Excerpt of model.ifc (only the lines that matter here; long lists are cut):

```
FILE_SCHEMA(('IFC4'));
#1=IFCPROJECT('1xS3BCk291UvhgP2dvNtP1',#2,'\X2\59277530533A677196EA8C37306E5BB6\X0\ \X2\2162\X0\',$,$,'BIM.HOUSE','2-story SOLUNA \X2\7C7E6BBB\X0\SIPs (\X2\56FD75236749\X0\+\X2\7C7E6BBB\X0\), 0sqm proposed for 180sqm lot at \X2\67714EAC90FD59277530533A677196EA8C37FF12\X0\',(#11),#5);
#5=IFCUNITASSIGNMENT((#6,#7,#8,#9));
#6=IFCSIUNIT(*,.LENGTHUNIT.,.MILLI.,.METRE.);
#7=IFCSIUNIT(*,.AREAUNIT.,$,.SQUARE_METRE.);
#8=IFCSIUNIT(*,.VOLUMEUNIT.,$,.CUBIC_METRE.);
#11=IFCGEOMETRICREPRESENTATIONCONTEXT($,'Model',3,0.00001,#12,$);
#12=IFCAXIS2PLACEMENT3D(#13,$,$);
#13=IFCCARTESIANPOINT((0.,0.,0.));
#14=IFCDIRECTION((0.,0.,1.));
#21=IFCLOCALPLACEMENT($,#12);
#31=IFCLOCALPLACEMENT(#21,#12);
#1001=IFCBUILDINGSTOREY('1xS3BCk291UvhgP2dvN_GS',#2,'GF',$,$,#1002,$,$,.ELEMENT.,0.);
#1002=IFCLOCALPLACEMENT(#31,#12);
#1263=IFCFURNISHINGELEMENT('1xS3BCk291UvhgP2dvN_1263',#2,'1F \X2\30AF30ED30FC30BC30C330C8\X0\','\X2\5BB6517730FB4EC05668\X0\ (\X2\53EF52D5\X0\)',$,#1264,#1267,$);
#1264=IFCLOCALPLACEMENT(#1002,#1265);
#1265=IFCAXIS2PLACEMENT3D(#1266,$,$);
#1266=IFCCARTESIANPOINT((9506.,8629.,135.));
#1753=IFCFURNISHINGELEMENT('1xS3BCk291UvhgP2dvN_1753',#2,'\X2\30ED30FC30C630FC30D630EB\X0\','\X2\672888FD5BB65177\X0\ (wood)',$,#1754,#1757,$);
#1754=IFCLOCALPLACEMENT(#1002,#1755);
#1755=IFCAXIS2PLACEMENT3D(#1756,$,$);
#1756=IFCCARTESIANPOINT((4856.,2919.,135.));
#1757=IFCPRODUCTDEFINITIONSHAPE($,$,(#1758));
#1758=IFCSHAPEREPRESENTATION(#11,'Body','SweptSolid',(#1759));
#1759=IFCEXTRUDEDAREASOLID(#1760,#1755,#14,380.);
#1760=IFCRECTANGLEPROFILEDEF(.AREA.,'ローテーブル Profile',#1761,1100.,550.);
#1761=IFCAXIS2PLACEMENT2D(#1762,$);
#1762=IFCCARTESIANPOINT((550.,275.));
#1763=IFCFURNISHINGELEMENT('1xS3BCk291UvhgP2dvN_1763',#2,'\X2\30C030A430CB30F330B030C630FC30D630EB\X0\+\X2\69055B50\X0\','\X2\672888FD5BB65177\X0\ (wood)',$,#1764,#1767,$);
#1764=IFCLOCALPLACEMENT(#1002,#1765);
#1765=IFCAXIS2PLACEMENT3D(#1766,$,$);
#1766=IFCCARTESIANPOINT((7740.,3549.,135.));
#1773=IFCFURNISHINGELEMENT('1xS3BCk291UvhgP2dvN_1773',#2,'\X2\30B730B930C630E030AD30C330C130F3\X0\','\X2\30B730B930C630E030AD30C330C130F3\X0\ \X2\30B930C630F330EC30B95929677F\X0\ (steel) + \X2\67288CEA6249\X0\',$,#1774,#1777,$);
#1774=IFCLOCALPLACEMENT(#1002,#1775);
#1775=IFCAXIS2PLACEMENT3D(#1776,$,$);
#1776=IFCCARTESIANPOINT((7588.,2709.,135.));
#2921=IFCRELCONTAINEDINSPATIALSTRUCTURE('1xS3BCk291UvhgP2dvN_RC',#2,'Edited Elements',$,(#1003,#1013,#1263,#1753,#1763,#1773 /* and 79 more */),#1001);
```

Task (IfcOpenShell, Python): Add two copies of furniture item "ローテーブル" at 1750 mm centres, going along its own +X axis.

```python
import ifcopenshell
import ifcopenshell.api.geometry
import ifcopenshell.api.root
import ifcopenshell.util.element
import ifcopenshell.util.placement
import ifcopenshell.util.unit

model = ifcopenshell.open("model.ifc")
unit_scale = ifcopenshell.util.unit.calculate_unit_scale(model)


def reuse_history(source, copy):
    """copy_class also copies each property set's owner history, people and application; keep the originals."""
    for rel in copy.IsDefinedBy:
        if rel.is_a("IfcRelDefinesByProperties") and (history := rel.RelatingPropertyDefinition.OwnerHistory):
            rel.RelatingPropertyDefinition.OwnerHistory = source.OwnerHistory
            ifcopenshell.util.element.remove_deep2(model, history)


source = model.by_id(1753)
base = ifcopenshell.util.placement.get_local_placement(source.ObjectPlacement)
step = base[:3, 0] * 1.75 / unit_scale

for i in range(1, 3):
    copy = ifcopenshell.api.root.copy_class(model, product=source)
    copy.Representation = ifcopenshell.util.element.copy_deep(
        model, source.Representation, exclude=["IfcGeometricRepresentationContext", "IfcRepresentationMap"]
    )
    reuse_history(source, copy)
    matrix = base.copy()
    matrix[:3, 3] += i * step
    print("added at", matrix[:3, 3].round(3) + 0.0)
    ifcopenshell.api.geometry.edit_object_placement(model, product=copy, matrix=matrix, is_si=False)

model.write("model_edited.ifc")
```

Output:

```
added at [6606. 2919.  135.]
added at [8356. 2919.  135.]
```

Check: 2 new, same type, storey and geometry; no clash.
